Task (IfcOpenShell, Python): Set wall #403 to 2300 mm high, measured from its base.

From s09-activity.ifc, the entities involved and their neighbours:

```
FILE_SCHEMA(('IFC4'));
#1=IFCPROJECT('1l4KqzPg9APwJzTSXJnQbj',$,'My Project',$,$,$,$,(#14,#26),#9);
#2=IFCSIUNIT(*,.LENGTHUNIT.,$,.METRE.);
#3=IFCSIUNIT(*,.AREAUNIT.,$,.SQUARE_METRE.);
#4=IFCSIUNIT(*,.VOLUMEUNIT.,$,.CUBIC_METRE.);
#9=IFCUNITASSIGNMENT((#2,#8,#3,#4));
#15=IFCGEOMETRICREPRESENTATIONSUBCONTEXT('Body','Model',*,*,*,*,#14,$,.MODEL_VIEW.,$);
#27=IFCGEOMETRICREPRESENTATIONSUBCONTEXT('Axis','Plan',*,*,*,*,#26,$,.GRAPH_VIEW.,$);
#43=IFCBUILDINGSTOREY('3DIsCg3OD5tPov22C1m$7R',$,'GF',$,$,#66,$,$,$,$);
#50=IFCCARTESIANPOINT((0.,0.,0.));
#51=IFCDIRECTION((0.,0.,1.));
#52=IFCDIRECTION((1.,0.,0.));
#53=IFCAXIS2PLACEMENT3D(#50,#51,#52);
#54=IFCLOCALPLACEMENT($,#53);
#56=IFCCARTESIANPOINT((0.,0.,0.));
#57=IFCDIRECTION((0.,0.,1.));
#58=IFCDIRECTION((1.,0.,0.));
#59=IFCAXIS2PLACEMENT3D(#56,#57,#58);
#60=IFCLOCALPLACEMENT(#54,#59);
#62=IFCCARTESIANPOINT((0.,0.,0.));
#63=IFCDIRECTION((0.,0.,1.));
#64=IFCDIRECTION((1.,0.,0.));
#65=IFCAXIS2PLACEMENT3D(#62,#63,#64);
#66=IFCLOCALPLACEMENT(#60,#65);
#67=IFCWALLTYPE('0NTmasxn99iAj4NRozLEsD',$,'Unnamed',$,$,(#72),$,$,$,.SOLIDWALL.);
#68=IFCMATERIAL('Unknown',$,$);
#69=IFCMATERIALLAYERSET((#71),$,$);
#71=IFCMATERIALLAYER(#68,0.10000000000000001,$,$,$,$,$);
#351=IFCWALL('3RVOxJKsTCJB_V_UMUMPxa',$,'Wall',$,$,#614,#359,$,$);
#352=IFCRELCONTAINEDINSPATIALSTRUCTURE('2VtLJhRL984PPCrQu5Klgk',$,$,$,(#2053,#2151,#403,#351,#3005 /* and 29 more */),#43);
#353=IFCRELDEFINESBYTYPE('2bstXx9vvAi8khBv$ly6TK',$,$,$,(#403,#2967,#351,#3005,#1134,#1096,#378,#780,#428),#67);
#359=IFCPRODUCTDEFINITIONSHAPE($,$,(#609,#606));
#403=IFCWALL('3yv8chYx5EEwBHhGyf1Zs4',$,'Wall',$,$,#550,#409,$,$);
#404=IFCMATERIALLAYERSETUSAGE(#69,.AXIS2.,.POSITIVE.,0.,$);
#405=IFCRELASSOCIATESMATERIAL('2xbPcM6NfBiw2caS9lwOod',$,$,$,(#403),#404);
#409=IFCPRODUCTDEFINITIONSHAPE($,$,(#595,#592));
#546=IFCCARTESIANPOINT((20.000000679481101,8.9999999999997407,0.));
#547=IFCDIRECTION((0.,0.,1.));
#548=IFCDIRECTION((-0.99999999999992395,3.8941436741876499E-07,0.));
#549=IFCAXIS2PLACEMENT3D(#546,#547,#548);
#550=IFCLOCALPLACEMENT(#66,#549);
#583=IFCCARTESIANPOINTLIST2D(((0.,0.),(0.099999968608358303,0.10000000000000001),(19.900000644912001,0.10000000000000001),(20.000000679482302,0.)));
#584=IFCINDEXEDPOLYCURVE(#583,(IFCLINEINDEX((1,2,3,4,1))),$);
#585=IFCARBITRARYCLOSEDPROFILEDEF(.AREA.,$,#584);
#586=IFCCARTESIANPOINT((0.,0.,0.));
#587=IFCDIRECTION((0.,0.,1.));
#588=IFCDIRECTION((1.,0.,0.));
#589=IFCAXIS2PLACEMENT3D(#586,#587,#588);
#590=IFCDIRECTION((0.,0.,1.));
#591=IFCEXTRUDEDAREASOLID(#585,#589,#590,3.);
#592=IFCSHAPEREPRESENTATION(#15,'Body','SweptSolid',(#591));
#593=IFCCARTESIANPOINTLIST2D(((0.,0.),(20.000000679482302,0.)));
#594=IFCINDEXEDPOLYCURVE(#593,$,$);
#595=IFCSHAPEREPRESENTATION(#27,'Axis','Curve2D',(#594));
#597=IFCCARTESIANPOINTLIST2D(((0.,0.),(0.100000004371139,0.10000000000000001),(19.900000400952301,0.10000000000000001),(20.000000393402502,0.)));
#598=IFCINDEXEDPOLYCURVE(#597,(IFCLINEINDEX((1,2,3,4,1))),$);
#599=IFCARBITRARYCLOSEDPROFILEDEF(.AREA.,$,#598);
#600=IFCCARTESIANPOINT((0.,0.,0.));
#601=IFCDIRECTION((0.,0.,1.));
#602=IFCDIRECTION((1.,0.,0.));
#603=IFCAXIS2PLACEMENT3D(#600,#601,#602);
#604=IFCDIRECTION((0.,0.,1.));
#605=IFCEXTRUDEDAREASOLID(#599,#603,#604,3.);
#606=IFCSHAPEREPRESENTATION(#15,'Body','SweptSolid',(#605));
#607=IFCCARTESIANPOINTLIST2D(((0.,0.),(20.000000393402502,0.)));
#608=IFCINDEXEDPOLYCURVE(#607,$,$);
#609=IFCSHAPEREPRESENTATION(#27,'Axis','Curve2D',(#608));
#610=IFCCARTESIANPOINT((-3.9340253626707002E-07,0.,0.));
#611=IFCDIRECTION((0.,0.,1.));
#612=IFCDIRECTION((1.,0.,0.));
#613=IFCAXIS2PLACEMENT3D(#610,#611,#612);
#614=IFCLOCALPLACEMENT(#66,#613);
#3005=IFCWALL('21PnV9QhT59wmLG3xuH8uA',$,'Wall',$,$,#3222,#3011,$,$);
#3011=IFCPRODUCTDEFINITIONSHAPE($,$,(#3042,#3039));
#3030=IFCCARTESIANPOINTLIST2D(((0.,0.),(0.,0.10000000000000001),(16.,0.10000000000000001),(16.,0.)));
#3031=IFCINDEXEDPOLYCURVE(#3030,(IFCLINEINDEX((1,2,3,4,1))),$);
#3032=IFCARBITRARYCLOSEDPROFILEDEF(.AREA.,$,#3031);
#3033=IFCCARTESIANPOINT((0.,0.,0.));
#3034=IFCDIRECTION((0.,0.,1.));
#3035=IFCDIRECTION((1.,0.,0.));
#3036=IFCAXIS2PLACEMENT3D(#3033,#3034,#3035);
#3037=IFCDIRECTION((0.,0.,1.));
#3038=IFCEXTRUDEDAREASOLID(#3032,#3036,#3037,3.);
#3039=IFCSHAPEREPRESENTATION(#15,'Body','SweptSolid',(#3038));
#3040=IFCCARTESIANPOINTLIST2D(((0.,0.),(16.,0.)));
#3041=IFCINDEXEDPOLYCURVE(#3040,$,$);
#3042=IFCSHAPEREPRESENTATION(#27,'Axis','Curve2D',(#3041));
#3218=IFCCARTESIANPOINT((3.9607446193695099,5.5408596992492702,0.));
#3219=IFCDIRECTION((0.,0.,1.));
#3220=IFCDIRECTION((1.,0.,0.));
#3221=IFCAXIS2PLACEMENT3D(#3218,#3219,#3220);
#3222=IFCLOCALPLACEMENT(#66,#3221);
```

```python
import ifcopenshell
import ifcopenshell.geom
import ifcopenshell.util.representation
import ifcopenshell.util.shape
import ifcopenshell.util.unit

model = ifcopenshell.open("s09-activity.ifc")
unit_scale = ifcopenshell.util.unit.calculate_unit_scale(model)
settings = ifcopenshell.geom.settings()


def volume(element):
    """Net volume in cubic metres, openings subtracted."""
    shape = ifcopenshell.geom.create_shape(settings, element)
    return ifcopenshell.util.shape.get_volume(shape.geometry)


wall = model.by_id(403)
before = volume(wall)

body = ifcopenshell.util.representation.get_representation(wall, "Model", "Body")
solid = body.Items[0]
old_height = solid.Depth
solid.Depth = 2.3 / unit_scale
after = volume(wall)

print(f"height {old_height:g} -> {solid.Depth:g}, volume {before:.3f} -> {after:.3f} m3")

model.write("s09-activity_rev.ifc")
```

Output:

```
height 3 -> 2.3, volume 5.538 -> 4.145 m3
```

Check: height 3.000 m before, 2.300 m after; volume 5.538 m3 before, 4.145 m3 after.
